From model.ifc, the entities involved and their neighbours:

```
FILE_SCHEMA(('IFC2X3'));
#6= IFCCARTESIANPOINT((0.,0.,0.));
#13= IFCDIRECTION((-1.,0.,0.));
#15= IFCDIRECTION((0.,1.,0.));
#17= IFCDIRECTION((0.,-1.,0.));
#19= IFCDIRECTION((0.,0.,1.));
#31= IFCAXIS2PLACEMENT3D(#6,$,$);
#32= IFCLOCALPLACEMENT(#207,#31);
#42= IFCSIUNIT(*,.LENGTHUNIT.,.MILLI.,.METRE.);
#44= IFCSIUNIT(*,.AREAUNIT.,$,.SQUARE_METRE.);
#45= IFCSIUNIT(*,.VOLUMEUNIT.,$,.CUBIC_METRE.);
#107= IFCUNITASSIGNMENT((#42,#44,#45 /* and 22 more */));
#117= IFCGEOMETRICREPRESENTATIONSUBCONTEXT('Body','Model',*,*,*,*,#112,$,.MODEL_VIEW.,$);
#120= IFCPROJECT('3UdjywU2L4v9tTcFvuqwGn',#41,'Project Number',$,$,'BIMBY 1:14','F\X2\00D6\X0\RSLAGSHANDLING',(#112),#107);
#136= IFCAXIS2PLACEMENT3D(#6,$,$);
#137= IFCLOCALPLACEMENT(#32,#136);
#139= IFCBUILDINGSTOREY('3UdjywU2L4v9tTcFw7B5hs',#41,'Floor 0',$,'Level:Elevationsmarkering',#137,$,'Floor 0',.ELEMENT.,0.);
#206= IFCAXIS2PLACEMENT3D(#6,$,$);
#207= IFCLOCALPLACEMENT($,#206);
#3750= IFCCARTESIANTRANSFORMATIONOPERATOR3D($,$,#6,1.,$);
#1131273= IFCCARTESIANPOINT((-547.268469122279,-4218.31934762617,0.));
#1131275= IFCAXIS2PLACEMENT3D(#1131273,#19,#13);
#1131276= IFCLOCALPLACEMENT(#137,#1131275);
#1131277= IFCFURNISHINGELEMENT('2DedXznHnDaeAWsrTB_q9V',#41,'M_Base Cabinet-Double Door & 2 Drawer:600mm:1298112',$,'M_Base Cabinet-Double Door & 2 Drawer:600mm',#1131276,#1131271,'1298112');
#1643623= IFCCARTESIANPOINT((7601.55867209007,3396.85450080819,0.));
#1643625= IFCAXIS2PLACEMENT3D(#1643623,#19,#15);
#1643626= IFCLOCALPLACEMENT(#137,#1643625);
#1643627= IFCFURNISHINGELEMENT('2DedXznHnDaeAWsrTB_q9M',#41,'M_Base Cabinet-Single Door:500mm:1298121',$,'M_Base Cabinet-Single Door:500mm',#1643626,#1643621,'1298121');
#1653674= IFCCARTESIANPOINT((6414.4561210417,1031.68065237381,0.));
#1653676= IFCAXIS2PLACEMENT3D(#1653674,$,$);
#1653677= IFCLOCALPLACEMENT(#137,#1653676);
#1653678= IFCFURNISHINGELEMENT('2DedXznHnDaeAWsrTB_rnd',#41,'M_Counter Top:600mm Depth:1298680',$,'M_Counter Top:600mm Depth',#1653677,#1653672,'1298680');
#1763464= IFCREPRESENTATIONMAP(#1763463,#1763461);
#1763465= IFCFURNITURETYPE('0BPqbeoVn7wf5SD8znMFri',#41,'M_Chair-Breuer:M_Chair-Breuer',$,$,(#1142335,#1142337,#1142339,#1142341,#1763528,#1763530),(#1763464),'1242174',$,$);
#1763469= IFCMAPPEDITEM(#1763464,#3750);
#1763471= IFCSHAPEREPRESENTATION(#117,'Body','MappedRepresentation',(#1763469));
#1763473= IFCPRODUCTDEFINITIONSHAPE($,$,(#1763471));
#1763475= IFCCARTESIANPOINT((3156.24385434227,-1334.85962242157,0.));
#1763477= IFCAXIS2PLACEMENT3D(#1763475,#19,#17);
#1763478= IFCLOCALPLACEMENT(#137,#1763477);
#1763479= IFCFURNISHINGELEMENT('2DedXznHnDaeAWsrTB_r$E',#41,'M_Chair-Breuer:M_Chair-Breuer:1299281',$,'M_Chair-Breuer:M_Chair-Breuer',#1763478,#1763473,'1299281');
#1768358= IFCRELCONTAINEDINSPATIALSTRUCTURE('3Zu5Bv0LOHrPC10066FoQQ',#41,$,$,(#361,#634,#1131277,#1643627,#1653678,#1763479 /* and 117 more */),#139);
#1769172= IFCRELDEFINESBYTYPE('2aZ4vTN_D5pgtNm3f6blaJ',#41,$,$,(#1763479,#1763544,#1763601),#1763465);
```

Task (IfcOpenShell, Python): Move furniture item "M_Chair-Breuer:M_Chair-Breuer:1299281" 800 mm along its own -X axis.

```python
import ifcopenshell
import ifcopenshell.api.geometry
import ifcopenshell.util.placement
import ifcopenshell.util.unit

model = ifcopenshell.open("model.ifc")
unit_scale = ifcopenshell.util.unit.calculate_unit_scale(model)

item = model.by_guid("2DedXznHnDaeAWsrTB_r$E")
matrix = ifcopenshell.util.placement.get_local_placement(item.ObjectPlacement)
matrix[:3, 3] -= matrix[:3, 0] * 0.8 / unit_scale
ifcopenshell.api.geometry.edit_object_placement(model, product=item, matrix=matrix, is_si=False)

print(ifcopenshell.util.placement.get_local_placement(item.ObjectPlacement).round(3) + 0.0)

model.write("model_edited.ifc")
```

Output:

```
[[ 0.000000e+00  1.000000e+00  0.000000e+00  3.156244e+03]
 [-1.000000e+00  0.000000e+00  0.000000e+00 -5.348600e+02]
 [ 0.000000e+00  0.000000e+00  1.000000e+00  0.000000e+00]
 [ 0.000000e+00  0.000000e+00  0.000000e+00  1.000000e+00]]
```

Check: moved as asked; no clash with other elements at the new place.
